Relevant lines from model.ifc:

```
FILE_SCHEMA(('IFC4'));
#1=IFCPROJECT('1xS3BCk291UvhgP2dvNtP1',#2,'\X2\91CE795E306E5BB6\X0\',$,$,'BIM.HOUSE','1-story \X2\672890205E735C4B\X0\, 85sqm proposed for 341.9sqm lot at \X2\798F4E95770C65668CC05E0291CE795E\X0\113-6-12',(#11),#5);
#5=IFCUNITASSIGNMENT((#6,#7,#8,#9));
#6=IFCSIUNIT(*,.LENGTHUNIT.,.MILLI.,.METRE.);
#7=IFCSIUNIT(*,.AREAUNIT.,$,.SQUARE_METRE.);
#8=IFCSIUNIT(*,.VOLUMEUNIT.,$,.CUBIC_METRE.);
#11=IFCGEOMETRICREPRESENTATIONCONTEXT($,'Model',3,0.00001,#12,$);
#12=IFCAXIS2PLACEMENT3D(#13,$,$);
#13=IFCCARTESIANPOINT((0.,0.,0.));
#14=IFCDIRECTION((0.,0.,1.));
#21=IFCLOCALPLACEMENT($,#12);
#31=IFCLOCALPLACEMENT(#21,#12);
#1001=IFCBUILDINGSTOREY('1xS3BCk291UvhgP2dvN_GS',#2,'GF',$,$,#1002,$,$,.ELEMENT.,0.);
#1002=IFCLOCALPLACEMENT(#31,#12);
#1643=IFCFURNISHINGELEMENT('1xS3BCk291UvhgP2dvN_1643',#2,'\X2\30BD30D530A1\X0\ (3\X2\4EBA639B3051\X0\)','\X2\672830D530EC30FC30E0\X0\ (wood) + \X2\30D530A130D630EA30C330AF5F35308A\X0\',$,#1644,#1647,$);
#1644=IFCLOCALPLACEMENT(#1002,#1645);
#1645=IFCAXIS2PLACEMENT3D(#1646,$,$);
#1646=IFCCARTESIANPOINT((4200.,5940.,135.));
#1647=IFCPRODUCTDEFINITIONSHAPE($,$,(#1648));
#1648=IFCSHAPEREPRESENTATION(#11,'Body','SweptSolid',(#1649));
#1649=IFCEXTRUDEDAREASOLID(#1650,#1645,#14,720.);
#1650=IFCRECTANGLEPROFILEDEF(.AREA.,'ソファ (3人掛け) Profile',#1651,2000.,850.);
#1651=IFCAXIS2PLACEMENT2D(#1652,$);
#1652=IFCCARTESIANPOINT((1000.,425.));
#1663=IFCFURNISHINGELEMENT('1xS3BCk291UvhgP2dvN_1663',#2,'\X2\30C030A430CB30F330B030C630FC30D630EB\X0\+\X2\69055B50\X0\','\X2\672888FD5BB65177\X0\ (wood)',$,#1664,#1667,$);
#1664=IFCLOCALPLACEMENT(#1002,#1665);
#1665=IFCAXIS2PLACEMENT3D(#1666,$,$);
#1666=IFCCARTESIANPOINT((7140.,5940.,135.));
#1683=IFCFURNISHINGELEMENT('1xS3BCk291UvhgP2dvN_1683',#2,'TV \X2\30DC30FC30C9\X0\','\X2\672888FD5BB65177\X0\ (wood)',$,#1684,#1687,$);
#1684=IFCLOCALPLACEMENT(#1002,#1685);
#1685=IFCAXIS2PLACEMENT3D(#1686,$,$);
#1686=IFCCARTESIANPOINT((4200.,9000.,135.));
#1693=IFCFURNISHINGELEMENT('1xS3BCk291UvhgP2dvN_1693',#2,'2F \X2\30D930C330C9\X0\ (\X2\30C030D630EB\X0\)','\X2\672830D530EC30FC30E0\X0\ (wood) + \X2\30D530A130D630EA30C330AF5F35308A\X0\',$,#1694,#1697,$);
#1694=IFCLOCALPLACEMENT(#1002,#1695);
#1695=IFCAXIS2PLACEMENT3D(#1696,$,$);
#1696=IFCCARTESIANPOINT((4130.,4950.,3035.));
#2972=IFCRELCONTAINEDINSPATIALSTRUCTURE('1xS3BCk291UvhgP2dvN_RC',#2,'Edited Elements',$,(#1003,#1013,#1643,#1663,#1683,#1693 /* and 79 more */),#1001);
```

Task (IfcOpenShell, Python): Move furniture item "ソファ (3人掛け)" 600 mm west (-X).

```python
import ifcopenshell
import ifcopenshell.api.geometry
import ifcopenshell.util.placement

model = ifcopenshell.open("model.ifc")

item = model.by_guid("1xS3BCk291UvhgP2dvN_1643")
matrix = ifcopenshell.util.placement.get_local_placement(item.ObjectPlacement)
matrix[0, 3] -= 600.0
ifcopenshell.api.geometry.edit_object_placement(model, product=item, matrix=matrix, is_si=False)

print(ifcopenshell.util.placement.get_local_placement(item.ObjectPlacement).round(3) + 0.0)

model.write("model_edited.ifc")
```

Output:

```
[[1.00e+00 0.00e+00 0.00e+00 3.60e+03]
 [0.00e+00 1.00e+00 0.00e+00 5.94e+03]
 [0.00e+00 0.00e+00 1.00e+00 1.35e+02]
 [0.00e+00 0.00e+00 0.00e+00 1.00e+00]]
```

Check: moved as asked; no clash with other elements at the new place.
